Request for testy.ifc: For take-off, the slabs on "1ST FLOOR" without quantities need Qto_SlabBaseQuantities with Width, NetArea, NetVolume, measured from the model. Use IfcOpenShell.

First a look at what the model holds.

```python
import ifcopenshell
import ifcopenshell.util.element
import ifcopenshell.util.unit

model = ifcopenshell.open("testy.ifc")
print(model.schema)
for unit_type in ("LENGTHUNIT", "AREAUNIT", "VOLUMEUNIT"):
    print(unit_type, ifcopenshell.util.unit.calculate_unit_scale(model, unit_type))
storey = next(s for s in model.by_type("IfcBuildingStorey") if s.Name == "1ST FLOOR")
slabs = [e for e in ifcopenshell.util.element.get_decomposition(storey) if e.is_a("IfcSlab")]
for e in sorted(slabs, key=lambda e: e.id()):
    print(e.id(), e.is_a(), e.Name, list(ifcopenshell.util.element.get_psets(e, qtos_only=True)), sep=" | ")
```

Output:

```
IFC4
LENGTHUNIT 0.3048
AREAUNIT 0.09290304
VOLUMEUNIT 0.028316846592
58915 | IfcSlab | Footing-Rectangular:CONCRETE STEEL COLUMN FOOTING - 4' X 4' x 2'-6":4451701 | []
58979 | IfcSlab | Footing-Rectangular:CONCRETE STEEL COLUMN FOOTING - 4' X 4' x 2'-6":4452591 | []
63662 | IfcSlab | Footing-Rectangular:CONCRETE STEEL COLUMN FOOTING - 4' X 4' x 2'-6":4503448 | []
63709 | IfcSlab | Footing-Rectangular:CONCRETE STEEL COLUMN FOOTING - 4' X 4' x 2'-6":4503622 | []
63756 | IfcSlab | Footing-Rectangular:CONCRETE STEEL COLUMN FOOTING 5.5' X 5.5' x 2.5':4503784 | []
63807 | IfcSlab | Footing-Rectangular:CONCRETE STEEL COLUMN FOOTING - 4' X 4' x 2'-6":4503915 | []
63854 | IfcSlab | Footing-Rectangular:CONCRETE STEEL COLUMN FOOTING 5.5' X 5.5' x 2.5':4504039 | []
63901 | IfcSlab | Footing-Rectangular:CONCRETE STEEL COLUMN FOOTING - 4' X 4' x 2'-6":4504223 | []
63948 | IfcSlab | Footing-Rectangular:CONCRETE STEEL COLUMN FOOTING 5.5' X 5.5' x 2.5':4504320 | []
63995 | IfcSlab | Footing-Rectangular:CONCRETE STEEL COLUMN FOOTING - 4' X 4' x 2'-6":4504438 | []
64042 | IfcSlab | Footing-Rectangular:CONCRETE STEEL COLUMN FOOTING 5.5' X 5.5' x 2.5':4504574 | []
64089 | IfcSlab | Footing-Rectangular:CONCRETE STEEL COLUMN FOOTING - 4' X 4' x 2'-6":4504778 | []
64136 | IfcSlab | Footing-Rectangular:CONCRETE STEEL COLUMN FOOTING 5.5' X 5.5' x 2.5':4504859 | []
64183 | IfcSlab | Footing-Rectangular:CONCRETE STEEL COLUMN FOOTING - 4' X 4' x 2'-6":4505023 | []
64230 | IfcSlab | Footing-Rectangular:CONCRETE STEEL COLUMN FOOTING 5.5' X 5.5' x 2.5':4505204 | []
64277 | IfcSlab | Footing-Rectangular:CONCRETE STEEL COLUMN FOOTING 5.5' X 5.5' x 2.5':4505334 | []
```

```python
import ifcopenshell
import ifcopenshell.api.pset
import ifcopenshell.geom
import ifcopenshell.util.element
import ifcopenshell.util.shape
import ifcopenshell.util.unit

model = ifcopenshell.open("testy.ifc")
unit_scale = ifcopenshell.util.unit.calculate_unit_scale(model)
area_scale = ifcopenshell.util.unit.calculate_unit_scale(model, "AREAUNIT")
volume_scale = ifcopenshell.util.unit.calculate_unit_scale(model, "VOLUMEUNIT")
settings = ifcopenshell.geom.settings()

storey = next(s for s in model.by_type("IfcBuildingStorey") if s.Name == "1ST FLOOR")
slabs = [e for e in ifcopenshell.util.element.get_decomposition(storey) if e.is_a("IfcSlab")]

for e in sorted(slabs, key=lambda e: e.id()):
    if ifcopenshell.util.element.get_psets(e, qtos_only=True, should_inherit=False):
        continue
    # Geometry comes back in metres, in the element's own axes.
    shape = ifcopenshell.geom.create_shape(settings, e)
    values = {
        "Width": ifcopenshell.util.shape.get_z(shape.geometry) / unit_scale,
        "NetArea": ifcopenshell.util.shape.get_footprint_area(shape.geometry) / area_scale,
        "NetVolume": ifcopenshell.util.shape.get_volume(shape.geometry) / volume_scale,
    }
    qto = ifcopenshell.api.pset.add_qto(model, product=e, name="Qto_SlabBaseQuantities")
    ifcopenshell.api.pset.edit_qto(model, qto=qto, properties=values)
    print(e.id(), {k: round(v, 3) for k, v in values.items()})

model.write("testy_v2.ifc")
```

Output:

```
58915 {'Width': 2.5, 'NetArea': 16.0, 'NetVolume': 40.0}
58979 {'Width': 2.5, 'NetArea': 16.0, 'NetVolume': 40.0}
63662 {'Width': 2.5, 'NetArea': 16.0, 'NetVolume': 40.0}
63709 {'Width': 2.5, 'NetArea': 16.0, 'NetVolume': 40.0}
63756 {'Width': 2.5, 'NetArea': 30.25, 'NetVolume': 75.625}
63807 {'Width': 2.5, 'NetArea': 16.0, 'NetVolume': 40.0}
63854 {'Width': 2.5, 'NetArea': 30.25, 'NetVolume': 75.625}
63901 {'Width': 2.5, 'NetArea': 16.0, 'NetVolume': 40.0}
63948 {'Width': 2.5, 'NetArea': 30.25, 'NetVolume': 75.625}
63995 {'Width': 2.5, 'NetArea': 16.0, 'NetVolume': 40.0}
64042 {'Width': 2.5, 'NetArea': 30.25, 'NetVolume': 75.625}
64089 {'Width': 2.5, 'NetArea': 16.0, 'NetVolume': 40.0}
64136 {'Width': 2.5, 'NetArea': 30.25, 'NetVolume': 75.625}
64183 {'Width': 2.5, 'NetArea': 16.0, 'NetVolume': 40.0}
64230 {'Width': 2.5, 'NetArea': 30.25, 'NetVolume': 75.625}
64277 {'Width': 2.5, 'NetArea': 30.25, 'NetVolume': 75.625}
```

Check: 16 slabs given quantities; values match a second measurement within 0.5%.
